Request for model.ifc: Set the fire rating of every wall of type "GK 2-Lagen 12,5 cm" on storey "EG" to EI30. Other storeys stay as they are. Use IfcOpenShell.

First a look at what the model holds.

```python
import ifcopenshell
import ifcopenshell.util.element

model = ifcopenshell.open("model.ifc")
print(model.schema)
storey = next(s for s in model.by_type("IfcBuildingStorey") if s.Name == "EG")
walls = [e for e in ifcopenshell.util.element.get_decomposition(storey) if e.is_a("IfcWall")]
seen = {}
for e in walls:
    element_type = ifcopenshell.util.element.get_type(e)
    key = (element_type.Name if element_type != e and element_type else None, ifcopenshell.util.element.get_pset(e, "Pset_WallCommon", "FireRating"))
    seen[key] = seen.get(key, 0) + 1
for (name, value), count in sorted(seen.items(), key=str):
    print(count, "x", name, "|", value)
```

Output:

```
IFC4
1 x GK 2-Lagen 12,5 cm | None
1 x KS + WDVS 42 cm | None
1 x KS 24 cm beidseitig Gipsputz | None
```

```python
import ifcopenshell
import ifcopenshell.api.pset
import ifcopenshell.util.element

model = ifcopenshell.open("model.ifc")

storey = next(s for s in model.by_type("IfcBuildingStorey") if s.Name == "EG")
walls = [e for e in ifcopenshell.util.element.get_decomposition(storey) if e.is_a("IfcWall")]

count = 0
for e in walls:
    element_type = ifcopenshell.util.element.get_type(e)
    if element_type in (None, e) or element_type.Name != "GK 2-Lagen 12,5 cm":
        continue
    # add_pset returns the element's existing set when there is one.
    pset = ifcopenshell.api.pset.add_pset(model, product=e, name="Pset_WallCommon")
    ifcopenshell.api.pset.edit_pset(model, pset=pset, properties={"FireRating": "EI30"})
    count += 1

print(count, "walls updated")

model.write("model-out.ifc")
```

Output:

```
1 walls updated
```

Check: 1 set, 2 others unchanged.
